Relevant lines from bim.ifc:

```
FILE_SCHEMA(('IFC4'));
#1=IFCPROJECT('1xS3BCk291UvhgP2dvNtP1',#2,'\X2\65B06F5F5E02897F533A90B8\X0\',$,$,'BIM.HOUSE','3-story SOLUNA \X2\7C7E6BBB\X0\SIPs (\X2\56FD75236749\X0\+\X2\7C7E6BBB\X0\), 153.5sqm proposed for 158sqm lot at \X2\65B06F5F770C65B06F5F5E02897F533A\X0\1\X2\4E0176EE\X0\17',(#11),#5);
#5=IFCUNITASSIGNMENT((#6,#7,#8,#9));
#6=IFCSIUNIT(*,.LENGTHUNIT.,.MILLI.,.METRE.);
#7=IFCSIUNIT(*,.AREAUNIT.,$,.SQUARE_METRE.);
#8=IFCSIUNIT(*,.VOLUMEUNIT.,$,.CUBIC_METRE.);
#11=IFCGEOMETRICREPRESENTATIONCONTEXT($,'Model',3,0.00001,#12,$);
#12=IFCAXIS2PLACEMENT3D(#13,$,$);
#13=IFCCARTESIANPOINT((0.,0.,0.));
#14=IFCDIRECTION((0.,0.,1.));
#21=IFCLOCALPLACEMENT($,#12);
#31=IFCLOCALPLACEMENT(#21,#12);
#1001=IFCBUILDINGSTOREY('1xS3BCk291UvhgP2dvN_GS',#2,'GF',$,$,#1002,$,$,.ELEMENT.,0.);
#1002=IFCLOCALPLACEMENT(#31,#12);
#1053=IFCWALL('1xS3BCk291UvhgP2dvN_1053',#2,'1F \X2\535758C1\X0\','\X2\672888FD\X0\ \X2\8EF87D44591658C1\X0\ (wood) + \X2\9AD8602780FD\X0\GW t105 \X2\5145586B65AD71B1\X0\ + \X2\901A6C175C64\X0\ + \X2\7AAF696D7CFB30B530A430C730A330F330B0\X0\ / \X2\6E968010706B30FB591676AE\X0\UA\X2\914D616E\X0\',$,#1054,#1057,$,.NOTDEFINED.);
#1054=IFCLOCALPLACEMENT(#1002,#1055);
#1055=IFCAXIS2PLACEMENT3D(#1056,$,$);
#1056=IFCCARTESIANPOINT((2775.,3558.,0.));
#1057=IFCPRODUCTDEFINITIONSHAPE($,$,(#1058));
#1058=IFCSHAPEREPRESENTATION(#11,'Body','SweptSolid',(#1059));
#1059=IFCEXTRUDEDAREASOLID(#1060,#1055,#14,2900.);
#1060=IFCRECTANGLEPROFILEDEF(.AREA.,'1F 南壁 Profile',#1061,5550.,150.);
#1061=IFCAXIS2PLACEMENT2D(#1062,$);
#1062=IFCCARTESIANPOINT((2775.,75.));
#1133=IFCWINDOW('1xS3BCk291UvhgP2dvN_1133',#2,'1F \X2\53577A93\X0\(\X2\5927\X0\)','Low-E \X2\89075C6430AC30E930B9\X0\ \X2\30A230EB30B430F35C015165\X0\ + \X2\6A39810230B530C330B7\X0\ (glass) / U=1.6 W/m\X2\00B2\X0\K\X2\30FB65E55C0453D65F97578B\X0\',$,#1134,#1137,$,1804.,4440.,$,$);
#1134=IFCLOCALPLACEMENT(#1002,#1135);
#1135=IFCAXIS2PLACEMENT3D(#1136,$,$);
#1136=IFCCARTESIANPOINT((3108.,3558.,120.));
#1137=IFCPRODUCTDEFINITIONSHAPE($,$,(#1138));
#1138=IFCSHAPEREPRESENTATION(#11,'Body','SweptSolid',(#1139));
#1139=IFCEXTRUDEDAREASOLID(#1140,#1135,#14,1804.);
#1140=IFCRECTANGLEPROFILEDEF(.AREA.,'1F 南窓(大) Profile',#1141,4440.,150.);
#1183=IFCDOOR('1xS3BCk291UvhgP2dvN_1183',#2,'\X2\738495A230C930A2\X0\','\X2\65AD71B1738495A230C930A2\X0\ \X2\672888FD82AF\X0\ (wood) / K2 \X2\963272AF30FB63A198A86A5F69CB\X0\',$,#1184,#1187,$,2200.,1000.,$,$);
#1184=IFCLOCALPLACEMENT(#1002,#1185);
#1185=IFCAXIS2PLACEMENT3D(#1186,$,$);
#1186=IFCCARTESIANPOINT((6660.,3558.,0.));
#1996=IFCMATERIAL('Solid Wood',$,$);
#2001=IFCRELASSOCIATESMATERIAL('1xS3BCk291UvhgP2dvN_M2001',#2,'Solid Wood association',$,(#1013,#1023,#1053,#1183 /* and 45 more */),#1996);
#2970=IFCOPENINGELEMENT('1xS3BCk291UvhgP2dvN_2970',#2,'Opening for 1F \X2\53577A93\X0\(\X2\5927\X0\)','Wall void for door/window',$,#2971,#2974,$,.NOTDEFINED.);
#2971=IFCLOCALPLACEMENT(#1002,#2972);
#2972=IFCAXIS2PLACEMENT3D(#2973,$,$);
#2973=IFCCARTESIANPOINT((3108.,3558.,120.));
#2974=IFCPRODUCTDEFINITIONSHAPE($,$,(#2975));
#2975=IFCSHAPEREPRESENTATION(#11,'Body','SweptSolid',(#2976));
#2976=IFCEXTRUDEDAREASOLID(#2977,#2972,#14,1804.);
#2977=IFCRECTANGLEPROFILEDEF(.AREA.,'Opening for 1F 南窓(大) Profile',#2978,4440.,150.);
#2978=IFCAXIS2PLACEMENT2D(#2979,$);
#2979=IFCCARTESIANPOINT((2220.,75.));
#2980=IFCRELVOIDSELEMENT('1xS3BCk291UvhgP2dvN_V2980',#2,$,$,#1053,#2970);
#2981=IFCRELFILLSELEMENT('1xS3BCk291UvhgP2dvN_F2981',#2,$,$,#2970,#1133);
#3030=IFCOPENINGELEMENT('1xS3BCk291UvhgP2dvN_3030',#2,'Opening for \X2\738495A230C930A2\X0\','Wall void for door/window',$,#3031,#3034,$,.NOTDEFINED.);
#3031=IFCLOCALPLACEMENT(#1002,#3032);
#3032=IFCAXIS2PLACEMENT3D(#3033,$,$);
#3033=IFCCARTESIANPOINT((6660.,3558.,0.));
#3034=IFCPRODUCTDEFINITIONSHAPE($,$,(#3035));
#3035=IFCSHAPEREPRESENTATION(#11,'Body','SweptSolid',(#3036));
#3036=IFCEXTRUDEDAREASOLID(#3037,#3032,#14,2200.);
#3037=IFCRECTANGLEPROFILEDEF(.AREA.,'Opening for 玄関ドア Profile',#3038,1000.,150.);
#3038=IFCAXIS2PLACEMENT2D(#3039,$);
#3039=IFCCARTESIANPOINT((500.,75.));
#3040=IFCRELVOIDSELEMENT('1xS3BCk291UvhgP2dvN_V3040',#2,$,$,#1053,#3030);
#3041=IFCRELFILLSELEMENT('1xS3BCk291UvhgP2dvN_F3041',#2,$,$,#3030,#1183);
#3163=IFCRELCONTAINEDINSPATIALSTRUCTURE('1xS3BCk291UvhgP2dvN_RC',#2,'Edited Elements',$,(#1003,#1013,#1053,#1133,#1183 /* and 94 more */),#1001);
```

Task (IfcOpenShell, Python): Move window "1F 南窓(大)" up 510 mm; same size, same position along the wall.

```python
import numpy as np
import ifcopenshell
import ifcopenshell.api.geometry
import ifcopenshell.util.placement
import ifcopenshell.util.unit

model = ifcopenshell.open("bim.ifc")
unit_scale = ifcopenshell.util.unit.calculate_unit_scale(model)

window = model.by_id(1133)
opening = window.FillsVoids[0].RelatingOpeningElement
dz = 0.51 / unit_scale

shift = np.array([0.0, 0.0, dz])
# The window is not placed relative to its opening, so move both.
for product in (opening, window):
    matrix = ifcopenshell.util.placement.get_local_placement(product.ObjectPlacement)
    matrix[:3, 3] += shift
    ifcopenshell.api.geometry.edit_object_placement(model, product=product, matrix=matrix, is_si=False)

print(f"moved by {dz * unit_scale:+.3f} m")

model.write("bim_v2.ifc")
```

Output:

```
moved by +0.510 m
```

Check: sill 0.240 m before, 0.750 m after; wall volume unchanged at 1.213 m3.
